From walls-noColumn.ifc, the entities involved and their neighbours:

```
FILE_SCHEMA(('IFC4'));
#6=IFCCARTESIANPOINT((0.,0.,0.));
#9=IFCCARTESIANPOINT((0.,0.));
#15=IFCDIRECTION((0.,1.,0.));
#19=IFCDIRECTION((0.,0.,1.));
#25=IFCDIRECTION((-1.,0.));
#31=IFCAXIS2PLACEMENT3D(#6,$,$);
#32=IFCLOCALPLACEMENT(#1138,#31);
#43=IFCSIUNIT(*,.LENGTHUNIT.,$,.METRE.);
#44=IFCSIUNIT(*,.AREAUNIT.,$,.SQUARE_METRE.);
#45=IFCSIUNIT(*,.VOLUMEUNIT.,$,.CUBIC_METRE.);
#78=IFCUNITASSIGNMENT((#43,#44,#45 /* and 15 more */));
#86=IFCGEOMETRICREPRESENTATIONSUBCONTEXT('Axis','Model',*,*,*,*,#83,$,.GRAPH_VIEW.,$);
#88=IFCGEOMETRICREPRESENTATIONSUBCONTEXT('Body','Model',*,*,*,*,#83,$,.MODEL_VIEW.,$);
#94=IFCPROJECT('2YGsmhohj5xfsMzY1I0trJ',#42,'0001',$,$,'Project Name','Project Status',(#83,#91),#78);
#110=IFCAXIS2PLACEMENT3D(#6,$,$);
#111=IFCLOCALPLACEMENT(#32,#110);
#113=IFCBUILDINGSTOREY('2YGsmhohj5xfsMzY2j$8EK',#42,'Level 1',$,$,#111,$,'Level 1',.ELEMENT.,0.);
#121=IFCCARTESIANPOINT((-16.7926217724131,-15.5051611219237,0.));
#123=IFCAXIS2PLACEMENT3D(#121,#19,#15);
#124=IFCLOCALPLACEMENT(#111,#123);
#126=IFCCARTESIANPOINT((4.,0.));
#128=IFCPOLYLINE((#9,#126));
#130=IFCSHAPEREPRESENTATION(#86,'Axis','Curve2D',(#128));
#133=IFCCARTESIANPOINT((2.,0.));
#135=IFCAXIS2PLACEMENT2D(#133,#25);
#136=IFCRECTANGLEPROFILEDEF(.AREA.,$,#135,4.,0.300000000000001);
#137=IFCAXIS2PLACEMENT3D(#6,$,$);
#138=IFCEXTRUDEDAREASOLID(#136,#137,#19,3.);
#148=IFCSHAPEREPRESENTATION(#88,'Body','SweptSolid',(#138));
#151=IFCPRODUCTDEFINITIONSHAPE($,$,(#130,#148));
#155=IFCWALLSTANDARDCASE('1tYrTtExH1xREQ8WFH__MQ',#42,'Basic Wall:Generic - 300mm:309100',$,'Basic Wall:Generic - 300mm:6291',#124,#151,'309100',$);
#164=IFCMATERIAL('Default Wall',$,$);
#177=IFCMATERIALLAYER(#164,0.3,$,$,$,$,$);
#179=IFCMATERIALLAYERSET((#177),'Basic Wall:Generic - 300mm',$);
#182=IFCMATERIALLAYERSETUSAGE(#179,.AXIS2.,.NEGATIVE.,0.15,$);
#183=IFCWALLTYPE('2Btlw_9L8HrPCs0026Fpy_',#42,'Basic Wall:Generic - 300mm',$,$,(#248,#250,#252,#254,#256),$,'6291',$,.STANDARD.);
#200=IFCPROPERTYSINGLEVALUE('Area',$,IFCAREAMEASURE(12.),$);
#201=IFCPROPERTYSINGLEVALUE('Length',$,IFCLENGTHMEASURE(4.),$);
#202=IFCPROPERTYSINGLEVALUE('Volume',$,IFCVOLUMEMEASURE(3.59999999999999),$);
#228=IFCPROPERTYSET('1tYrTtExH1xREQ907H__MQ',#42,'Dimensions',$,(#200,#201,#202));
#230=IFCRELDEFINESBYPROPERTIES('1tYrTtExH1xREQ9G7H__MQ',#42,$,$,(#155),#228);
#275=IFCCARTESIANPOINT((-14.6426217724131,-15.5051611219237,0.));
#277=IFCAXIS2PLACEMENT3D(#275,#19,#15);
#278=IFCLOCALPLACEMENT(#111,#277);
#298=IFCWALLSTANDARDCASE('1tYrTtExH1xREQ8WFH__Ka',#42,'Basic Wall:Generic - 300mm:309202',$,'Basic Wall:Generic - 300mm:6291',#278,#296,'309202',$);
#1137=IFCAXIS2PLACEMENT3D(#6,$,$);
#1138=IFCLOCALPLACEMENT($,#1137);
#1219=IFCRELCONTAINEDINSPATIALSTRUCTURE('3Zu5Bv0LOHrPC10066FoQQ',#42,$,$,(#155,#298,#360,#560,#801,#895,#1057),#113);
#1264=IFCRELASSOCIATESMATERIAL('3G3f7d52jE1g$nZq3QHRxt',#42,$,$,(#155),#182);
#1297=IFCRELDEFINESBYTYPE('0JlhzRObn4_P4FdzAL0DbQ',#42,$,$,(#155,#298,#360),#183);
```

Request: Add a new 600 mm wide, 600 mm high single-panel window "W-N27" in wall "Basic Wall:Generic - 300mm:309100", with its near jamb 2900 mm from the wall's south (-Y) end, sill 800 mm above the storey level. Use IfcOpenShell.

```python
import numpy as np
import ifcopenshell
import ifcopenshell.api.feature
import ifcopenshell.api.geometry
import ifcopenshell.api.pset
import ifcopenshell.api.root
import ifcopenshell.api.spatial
import ifcopenshell.geom
import ifcopenshell.util.element
import ifcopenshell.util.placement
import ifcopenshell.util.representation
import ifcopenshell.util.shape
import ifcopenshell.util.unit

model = ifcopenshell.open("walls-noColumn.ifc")
unit_scale = ifcopenshell.util.unit.calculate_unit_scale(model)
area_scale = ifcopenshell.util.unit.calculate_unit_scale(model, "AREAUNIT")
volume_scale = ifcopenshell.util.unit.calculate_unit_scale(model, "VOLUMEUNIT")
settings = ifcopenshell.geom.settings()


def volume(element):
    """Net volume in cubic metres, openings subtracted."""
    shape = ifcopenshell.geom.create_shape(settings, element)
    return ifcopenshell.util.shape.get_volume(shape.geometry)


wall = model.by_guid("1tYrTtExH1xREQ8WFH__MQ")
storey = ifcopenshell.util.element.get_container(wall, ifc_class="IfcBuildingStorey")
context = ifcopenshell.util.representation.get_context(model, "Model", "Body", "MODEL_VIEW")
before = volume(wall)

width, height, from_end, sill = 0.6, 0.6, 2.9, 0.8  # metres

# The wall runs along its own X axis, and the end named is its -X end.
wall_shape = ifcopenshell.geom.create_shape(settings, wall)
x, y, z = ifcopenshell.util.shape.get_vertices(wall_shape.geometry).T
start = x.min() + from_end
face, thickness = float(y.min()), float(y.max() - y.min())
wall_matrix = ifcopenshell.util.placement.get_local_placement(wall.ObjectPlacement)
level = ifcopenshell.util.placement.get_local_placement(storey.ObjectPlacement)[2, 3]


def in_wall(x, y):
    """Placement at x, y metres in the wall's axes, at sill height."""
    matrix = wall_matrix.copy()
    matrix[:, 3] = wall_matrix @ np.array([x / unit_scale, y / unit_scale, 0.0, 1.0])
    matrix[2, 3] = level + sill / unit_scale
    return matrix


# Opening: a box that overshoots both wall faces by 50 mm.
opening = ifcopenshell.api.root.create_entity(model, ifc_class="IfcOpeningElement", predefined_type="OPENING")
box = ifcopenshell.api.geometry.add_wall_representation(
    model, context=context, length=width, height=height, thickness=thickness + 0.1
)
ifcopenshell.api.geometry.assign_representation(model, product=opening, representation=box)
ifcopenshell.api.geometry.edit_object_placement(model, product=opening, matrix=in_wall(start, face - 0.05), is_si=False)
ifcopenshell.api.feature.add_feature(model, feature=opening, element=wall)

window = ifcopenshell.api.root.create_entity(model, ifc_class="IfcWindow", name="W-N27", predefined_type="WINDOW")
window.OverallWidth, window.OverallHeight = width / unit_scale, height / unit_scale
window.PartitioningType = "SINGLE_PANEL"
body = ifcopenshell.api.geometry.add_window_representation(
    model,
    context=context,
    overall_width=window.OverallWidth,
    overall_height=window.OverallHeight,
    partition_type="SINGLE_PANEL",
)
ifcopenshell.api.geometry.assign_representation(model, product=window, representation=body)
ifcopenshell.api.spatial.assign_container(model, products=[window], relating_structure=storey)
ifcopenshell.api.feature.add_filling(model, opening=opening, element=window)

# Centre the window in the wall's thickness.
ifcopenshell.api.geometry.edit_object_placement(model, product=window, matrix=in_wall(start, face), is_si=False)
window_shape = ifcopenshell.geom.create_shape(settings, window)
depth = ifcopenshell.util.shape.get_vertices(window_shape.geometry)[:, 1]
offset = face + thickness / 2 - (depth.min() + depth.max()) / 2
ifcopenshell.api.geometry.edit_object_placement(model, product=window, matrix=in_wall(start, offset), is_si=False)

after = volume(wall)

# Update the wall's stored quantities.
pset = model.by_id(ifcopenshell.util.element.get_pset(wall, "Dimensions", should_inherit=False)["id"])
ifcopenshell.api.pset.edit_pset(model, pset=pset, properties={
    "Area": model.create_entity("IfcAreaMeasure", after / thickness / area_scale),
    "Volume": model.create_entity("IfcVolumeMeasure", after / volume_scale),
})

print(f"wall volume {before:.3f} -> {after:.3f} m3")

model.write("walls-noColumn_edited.ifc")
```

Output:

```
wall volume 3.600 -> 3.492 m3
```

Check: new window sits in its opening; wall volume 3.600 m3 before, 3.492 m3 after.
